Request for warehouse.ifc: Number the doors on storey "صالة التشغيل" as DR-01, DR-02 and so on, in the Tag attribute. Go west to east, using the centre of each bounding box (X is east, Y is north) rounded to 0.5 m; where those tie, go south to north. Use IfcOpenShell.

First a look at what the model holds.

```python
import ifcopenshell
import ifcopenshell.util.element
import ifcopenshell.util.placement

model = ifcopenshell.open("warehouse.ifc")
print(model.schema)
storey = next(s for s in model.by_type("IfcBuildingStorey") if s.Name == "صالة التشغيل")
doors = [e for e in ifcopenshell.util.element.get_decomposition(storey) if e.is_a("IfcDoor")]
for e in sorted(doors, key=lambda e: e.id()):
    origin = ifcopenshell.util.placement.get_local_placement(e.ObjectPlacement)[:3, 3]
    print(e.id(), e.Tag, e.Name, origin.round(2) + 0.0, sep=" | ")
```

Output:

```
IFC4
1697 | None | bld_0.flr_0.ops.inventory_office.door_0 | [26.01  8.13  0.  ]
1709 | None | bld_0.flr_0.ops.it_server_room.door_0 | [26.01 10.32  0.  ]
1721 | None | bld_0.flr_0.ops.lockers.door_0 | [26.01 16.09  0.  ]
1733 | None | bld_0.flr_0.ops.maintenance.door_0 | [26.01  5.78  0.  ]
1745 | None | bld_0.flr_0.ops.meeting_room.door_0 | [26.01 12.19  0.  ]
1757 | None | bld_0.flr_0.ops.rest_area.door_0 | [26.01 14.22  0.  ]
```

```python
import ifcopenshell
import ifcopenshell.geom
import ifcopenshell.util.element
import ifcopenshell.util.shape

model = ifcopenshell.open("warehouse.ifc")
settings = ifcopenshell.geom.settings()
settings.set("use-world-coords", True)


def centre(element):
    shape = ifcopenshell.geom.create_shape(settings, element)
    return ifcopenshell.util.shape.get_bbox_centroid(shape.geometry)


storey = next(s for s in model.by_type("IfcBuildingStorey") if s.Name == "صالة التشغيل")
doors = [e for e in ifcopenshell.util.element.get_decomposition(storey) if e.is_a("IfcDoor")]

# Insertion points can sit at a corner or the storey origin, so sort by the geometry (in metres).
centres = {e: centre(e) for e in doors}
doors.sort(key=lambda e: (round(centres[e][0] / 0.5), centres[e][1]))

for i, e in enumerate(doors, start=1):
    number = f"DR-{i:02d}"
    e.Tag = number
    print(e.id(), number)

model.write("warehouse_rev.ifc")
```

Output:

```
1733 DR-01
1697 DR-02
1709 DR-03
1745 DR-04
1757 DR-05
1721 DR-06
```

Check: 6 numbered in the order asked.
